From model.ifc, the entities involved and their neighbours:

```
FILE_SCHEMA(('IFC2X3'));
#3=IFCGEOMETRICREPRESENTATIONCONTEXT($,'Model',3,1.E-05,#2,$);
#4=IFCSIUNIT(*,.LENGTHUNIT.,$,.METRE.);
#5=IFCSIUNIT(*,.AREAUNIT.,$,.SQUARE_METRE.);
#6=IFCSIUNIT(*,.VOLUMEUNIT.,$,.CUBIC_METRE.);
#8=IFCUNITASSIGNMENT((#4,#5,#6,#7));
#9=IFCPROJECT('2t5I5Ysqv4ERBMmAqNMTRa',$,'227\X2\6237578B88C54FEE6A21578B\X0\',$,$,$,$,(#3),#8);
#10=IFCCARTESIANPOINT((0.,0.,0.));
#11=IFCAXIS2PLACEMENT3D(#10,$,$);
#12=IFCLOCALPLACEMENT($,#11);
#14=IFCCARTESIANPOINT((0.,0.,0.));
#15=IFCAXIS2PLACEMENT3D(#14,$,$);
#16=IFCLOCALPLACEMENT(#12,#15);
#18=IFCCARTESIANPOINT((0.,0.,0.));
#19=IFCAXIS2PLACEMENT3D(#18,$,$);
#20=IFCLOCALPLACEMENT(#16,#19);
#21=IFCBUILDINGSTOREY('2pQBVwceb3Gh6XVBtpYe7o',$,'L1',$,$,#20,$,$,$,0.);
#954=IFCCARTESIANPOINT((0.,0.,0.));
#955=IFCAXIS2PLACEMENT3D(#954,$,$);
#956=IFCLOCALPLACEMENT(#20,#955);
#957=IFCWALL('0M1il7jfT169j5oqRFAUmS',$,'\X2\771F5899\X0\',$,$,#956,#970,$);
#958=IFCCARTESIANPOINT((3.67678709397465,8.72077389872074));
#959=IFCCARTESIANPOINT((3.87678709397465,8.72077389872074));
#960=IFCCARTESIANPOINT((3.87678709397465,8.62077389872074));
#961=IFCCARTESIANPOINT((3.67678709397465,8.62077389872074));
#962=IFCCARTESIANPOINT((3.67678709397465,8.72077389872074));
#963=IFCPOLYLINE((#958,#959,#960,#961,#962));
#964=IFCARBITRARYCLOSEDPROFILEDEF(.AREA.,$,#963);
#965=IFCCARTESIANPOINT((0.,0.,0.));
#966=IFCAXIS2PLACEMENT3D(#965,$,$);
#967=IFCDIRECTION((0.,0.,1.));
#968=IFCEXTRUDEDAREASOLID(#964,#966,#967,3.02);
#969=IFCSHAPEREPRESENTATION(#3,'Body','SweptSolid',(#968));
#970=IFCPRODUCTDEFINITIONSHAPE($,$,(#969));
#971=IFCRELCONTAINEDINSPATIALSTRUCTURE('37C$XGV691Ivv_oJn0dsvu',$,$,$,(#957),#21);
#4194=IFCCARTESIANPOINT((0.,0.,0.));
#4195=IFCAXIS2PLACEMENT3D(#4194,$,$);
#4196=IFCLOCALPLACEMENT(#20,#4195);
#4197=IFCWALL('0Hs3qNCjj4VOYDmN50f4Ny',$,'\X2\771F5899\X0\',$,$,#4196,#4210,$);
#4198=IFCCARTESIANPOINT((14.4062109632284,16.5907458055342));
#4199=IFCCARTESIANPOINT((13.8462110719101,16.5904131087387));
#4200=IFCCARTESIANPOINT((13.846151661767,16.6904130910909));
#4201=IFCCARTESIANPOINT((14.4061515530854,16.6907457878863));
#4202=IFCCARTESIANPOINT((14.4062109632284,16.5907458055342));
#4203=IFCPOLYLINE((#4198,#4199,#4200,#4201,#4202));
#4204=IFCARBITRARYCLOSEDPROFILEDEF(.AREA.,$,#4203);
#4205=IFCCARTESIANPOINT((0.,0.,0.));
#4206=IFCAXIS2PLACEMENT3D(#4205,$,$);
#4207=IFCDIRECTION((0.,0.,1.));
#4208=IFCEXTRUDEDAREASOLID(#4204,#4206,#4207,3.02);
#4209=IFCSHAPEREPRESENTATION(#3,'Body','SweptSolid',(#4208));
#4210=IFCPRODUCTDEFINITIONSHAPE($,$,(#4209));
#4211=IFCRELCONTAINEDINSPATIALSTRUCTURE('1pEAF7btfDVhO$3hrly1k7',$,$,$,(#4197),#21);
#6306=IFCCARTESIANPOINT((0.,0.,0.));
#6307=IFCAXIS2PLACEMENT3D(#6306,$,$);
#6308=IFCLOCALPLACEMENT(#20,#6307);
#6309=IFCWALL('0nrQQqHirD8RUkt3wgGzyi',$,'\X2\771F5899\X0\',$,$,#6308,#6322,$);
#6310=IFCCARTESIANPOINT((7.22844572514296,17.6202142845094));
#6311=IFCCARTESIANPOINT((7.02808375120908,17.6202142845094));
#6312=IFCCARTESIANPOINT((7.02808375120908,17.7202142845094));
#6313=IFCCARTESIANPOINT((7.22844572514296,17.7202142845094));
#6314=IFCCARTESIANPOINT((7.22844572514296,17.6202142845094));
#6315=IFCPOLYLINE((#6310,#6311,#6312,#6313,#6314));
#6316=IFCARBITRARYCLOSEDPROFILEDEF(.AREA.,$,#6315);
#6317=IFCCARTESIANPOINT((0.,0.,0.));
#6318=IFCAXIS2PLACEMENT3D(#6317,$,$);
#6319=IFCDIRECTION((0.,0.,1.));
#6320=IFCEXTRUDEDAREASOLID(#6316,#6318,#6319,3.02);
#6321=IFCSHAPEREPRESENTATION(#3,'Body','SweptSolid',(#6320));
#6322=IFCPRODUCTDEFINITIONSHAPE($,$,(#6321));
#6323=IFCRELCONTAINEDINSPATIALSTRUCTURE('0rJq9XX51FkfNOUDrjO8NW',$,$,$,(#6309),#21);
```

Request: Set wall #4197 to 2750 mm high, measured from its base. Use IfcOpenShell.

```python
import ifcopenshell
import ifcopenshell.geom
import ifcopenshell.util.shape
import ifcopenshell.util.unit

model = ifcopenshell.open("model.ifc")
unit_scale = ifcopenshell.util.unit.calculate_unit_scale(model)
settings = ifcopenshell.geom.settings()


def volume(element):
    """Net volume in cubic metres, openings subtracted."""
    shape = ifcopenshell.geom.create_shape(settings, element)
    return ifcopenshell.util.shape.get_volume(shape.geometry)


wall = model.by_guid("0Hs3qNCjj4VOYDmN50f4Ny")
before = volume(wall)

body = next(r for r in wall.Representation.Representations if r.RepresentationIdentifier == "Body")
solid = body.Items[0]
old_height = solid.Depth
solid.Depth = 2.75 / unit_scale
after = volume(wall)

print(f"height {old_height:g} -> {solid.Depth:g}, volume {before:.3f} -> {after:.3f} m3")

model.write("model_updated.ifc")
```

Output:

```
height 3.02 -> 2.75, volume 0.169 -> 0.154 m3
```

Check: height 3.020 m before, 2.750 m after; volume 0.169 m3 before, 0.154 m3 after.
